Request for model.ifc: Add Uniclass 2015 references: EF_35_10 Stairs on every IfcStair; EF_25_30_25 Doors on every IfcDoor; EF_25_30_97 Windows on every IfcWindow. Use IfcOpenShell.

First a look at what the model holds.

```python
import ifcopenshell

model = ifcopenshell.open("model.ifc")
print(model.schema)
print("classifications:", [c.Name for c in model.by_type("IfcClassification")])
for ifc_class in ("IfcDoor", "IfcRoof", "IfcStair", "IfcWall", "IfcWindow"):
    print(ifc_class, len(model.by_type(ifc_class)))
```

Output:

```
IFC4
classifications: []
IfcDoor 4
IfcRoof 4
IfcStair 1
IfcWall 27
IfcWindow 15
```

```python
import ifcopenshell
import ifcopenshell.api.classification

model = ifcopenshell.open("model.ifc")

system = ifcopenshell.api.classification.add_classification(model, classification="Uniclass 2015")

codes = {
    "IfcStair": ("EF_35_10", "Stairs"),
    "IfcDoor": ("EF_25_30_25", "Doors"),
    "IfcWindow": ("EF_25_30_97", "Windows"),
}
for ifc_class, (code, name) in codes.items():
    products = model.by_type(ifc_class)
    ifcopenshell.api.classification.add_reference(
        model, products=products, classification=system, identification=code, name=name
    )
    print(code, len(products))

model.write("model_edited.ifc")
```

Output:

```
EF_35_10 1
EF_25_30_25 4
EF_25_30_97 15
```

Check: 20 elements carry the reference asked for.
